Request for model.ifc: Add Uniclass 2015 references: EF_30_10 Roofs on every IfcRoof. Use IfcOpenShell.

First a look at what the model holds.

```python
import ifcopenshell

model = ifcopenshell.open("model.ifc")
print(model.schema)
print("classifications:", [c.Name for c in model.by_type("IfcClassification")])
for ifc_class in ("IfcDoor", "IfcRoof", "IfcStair", "IfcWall", "IfcWindow"):
    print(ifc_class, len(model.by_type(ifc_class)))
```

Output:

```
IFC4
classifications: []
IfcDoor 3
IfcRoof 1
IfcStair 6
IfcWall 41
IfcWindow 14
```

```python
import ifcopenshell
import ifcopenshell.api.classification

model = ifcopenshell.open("model.ifc")

system = ifcopenshell.api.classification.add_classification(model, classification="Uniclass 2015")

codes = {
    "IfcRoof": ("EF_30_10", "Roofs"),
}
for ifc_class, (code, name) in codes.items():
    products = model.by_type(ifc_class)
    ifcopenshell.api.classification.add_reference(
        model, products=products, classification=system, identification=code, name=name
    )
    print(code, len(products))

model.write("model-out.ifc")
```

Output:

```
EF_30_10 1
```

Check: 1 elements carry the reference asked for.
